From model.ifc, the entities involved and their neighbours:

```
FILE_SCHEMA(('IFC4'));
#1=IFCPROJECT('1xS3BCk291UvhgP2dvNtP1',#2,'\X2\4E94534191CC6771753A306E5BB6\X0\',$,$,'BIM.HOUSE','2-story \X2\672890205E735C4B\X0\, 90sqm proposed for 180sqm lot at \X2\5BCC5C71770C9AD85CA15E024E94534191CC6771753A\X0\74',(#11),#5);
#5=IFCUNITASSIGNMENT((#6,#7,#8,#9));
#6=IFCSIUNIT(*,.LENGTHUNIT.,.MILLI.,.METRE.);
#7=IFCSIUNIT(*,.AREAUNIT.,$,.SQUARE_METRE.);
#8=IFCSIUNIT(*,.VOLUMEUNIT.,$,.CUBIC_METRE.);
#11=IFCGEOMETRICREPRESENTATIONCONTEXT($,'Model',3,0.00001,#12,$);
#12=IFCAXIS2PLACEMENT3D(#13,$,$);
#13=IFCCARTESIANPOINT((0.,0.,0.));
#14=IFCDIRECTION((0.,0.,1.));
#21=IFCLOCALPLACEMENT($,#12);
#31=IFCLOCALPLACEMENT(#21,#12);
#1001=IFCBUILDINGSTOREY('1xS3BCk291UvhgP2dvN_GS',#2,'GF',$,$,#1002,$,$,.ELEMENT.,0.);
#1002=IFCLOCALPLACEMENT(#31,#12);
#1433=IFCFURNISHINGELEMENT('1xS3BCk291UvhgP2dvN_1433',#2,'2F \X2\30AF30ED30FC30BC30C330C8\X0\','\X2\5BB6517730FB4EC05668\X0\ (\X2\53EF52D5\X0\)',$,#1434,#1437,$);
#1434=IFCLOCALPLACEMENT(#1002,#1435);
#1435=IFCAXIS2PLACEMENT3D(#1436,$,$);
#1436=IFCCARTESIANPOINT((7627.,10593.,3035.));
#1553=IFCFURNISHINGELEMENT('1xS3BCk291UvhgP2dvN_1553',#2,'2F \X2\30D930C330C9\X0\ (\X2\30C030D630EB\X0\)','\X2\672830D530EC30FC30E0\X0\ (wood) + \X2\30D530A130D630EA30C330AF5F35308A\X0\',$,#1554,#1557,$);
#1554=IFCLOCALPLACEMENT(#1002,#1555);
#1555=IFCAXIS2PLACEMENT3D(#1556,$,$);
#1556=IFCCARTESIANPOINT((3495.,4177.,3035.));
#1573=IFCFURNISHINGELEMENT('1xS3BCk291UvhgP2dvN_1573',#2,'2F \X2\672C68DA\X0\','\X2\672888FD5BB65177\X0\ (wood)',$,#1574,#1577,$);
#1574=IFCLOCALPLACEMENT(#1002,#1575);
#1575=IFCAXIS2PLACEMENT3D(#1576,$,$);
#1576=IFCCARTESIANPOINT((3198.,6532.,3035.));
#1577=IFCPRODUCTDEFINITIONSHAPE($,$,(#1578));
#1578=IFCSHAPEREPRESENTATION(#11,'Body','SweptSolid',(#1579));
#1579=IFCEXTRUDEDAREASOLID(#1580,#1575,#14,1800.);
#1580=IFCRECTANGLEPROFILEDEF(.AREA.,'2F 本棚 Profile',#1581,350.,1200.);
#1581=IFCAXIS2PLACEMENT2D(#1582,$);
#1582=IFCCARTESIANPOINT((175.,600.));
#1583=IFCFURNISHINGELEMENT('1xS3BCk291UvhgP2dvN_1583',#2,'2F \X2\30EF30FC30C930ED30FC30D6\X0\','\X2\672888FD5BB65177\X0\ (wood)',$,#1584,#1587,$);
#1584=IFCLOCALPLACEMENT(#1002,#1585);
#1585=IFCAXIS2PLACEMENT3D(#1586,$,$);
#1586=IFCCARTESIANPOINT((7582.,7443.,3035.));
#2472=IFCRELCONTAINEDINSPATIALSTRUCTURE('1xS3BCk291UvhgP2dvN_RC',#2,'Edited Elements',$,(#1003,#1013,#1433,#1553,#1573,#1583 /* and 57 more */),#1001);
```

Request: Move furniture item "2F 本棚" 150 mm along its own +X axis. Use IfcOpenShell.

```python
import ifcopenshell
import ifcopenshell.api.geometry
import ifcopenshell.util.placement

model = ifcopenshell.open("model.ifc")

item = model.by_guid("1xS3BCk291UvhgP2dvN_1573")
matrix = ifcopenshell.util.placement.get_local_placement(item.ObjectPlacement)
matrix[:3, 3] += matrix[:3, 0] * 150.0
ifcopenshell.api.geometry.edit_object_placement(model, product=item, matrix=matrix, is_si=False)

print(ifcopenshell.util.placement.get_local_placement(item.ObjectPlacement).round(3) + 0.0)

model.write("model_edited.ifc")
```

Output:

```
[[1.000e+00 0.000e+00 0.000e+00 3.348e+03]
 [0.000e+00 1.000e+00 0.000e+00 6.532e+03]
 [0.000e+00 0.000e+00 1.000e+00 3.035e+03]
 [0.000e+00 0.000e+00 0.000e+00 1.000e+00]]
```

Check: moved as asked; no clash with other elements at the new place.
